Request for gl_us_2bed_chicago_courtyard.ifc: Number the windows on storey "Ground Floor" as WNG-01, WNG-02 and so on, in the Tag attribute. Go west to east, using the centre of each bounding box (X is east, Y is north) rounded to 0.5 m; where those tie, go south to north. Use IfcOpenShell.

First a look at what the model holds.

```python
import ifcopenshell
import ifcopenshell.util.element
import ifcopenshell.util.placement

model = ifcopenshell.open("gl_us_2bed_chicago_courtyard.ifc")
print(model.schema)
storey = next(s for s in model.by_type("IfcBuildingStorey") if s.Name == "Ground Floor")
windows = [e for e in ifcopenshell.util.element.get_decomposition(storey) if e.is_a("IfcWindow")]
for e in sorted(windows, key=lambda e: e.id()):
    origin = ifcopenshell.util.placement.get_local_placement(e.ObjectPlacement)[:3, 3]
    print(e.id(), e.Tag, e.Name, origin.round(2) + 0.0, sep=" | ")
```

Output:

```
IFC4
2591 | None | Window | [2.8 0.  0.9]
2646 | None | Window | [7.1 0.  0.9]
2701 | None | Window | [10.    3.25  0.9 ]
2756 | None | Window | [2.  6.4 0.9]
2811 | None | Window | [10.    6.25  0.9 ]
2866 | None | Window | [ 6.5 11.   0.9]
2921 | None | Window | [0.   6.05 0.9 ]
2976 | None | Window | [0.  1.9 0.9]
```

```python
import ifcopenshell
import ifcopenshell.geom
import ifcopenshell.util.element
import ifcopenshell.util.shape

model = ifcopenshell.open("gl_us_2bed_chicago_courtyard.ifc")
settings = ifcopenshell.geom.settings()
settings.set("use-world-coords", True)


def centre(element):
    shape = ifcopenshell.geom.create_shape(settings, element)
    return ifcopenshell.util.shape.get_bbox_centroid(shape.geometry)


storey = next(s for s in model.by_type("IfcBuildingStorey") if s.Name == "Ground Floor")
windows = [e for e in ifcopenshell.util.element.get_decomposition(storey) if e.is_a("IfcWindow")]

# Insertion points can sit at a corner or the storey origin, so sort by the geometry (in metres).
centres = {e: centre(e) for e in windows}
windows.sort(key=lambda e: (round(centres[e][0] / 0.5), centres[e][1]))

for i, e in enumerate(windows, start=1):
    number = f"WNG-{i:02d}"
    e.Tag = number
    print(e.id(), number)

model.write("gl_us_2bed_chicago_courtyard_updated.ifc")
```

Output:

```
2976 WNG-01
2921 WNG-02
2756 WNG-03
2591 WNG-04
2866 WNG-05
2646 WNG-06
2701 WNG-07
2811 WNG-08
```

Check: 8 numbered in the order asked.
